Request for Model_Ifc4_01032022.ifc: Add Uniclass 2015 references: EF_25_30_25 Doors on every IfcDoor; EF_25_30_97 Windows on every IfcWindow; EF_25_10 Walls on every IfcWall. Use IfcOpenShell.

First a look at what the model holds.

```python
import ifcopenshell

model = ifcopenshell.open("Model_Ifc4_01032022.ifc")
print(model.schema)
print("classifications:", [c.Name for c in model.by_type("IfcClassification")])
for ifc_class in ("IfcDoor", "IfcRoof", "IfcStair", "IfcWall", "IfcWindow"):
    print(ifc_class, len(model.by_type(ifc_class)))
```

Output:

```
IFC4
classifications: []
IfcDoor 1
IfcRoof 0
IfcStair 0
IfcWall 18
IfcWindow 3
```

```python
import ifcopenshell
import ifcopenshell.api.classification

model = ifcopenshell.open("Model_Ifc4_01032022.ifc")

system = ifcopenshell.api.classification.add_classification(model, classification="Uniclass 2015")

codes = {
    "IfcDoor": ("EF_25_30_25", "Doors"),
    "IfcWindow": ("EF_25_30_97", "Windows"),
    "IfcWall": ("EF_25_10", "Walls"),
}
for ifc_class, (code, name) in codes.items():
    products = model.by_type(ifc_class)
    ifcopenshell.api.classification.add_reference(
        model, products=products, classification=system, identification=code, name=name
    )
    print(code, len(products))

model.write("Model_Ifc4_01032022_edited.ifc")
```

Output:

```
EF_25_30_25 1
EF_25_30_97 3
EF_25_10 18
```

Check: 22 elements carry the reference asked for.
